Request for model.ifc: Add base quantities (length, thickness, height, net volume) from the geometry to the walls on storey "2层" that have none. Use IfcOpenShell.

First a look at what the model holds.

```python
import ifcopenshell
import ifcopenshell.util.element
import ifcopenshell.util.unit

model = ifcopenshell.open("model.ifc")
print(model.schema)
for unit_type in ("LENGTHUNIT", "AREAUNIT", "VOLUMEUNIT"):
    print(unit_type, ifcopenshell.util.unit.calculate_unit_scale(model, unit_type))
storey = next(s for s in model.by_type("IfcBuildingStorey") if s.Name == "2层")
walls = [e for e in ifcopenshell.util.element.get_decomposition(storey) if e.is_a("IfcWall")]
for e in sorted(walls, key=lambda e: e.id()):
    print(e.id(), e.is_a(), e.Name, list(ifcopenshell.util.element.get_psets(e, qtos_only=True)), sep=" | ")
```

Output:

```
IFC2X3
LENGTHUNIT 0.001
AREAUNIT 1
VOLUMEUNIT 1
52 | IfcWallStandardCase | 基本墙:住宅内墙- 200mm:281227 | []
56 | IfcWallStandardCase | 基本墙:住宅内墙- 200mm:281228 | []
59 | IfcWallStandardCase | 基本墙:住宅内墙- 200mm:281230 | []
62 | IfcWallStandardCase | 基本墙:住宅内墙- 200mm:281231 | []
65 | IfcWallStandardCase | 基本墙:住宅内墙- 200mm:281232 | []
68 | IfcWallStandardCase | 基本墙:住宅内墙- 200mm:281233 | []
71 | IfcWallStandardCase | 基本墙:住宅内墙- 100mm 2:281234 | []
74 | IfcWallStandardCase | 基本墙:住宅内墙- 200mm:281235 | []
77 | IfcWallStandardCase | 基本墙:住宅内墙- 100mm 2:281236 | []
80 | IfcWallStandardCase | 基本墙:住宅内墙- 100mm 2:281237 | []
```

```python
import ifcopenshell
import ifcopenshell.api.pset
import ifcopenshell.geom
import ifcopenshell.util.element
import ifcopenshell.util.shape
import ifcopenshell.util.unit

model = ifcopenshell.open("model.ifc")
unit_scale = ifcopenshell.util.unit.calculate_unit_scale(model)
volume_scale = ifcopenshell.util.unit.calculate_unit_scale(model, "VOLUMEUNIT")
settings = ifcopenshell.geom.settings()

storey = next(s for s in model.by_type("IfcBuildingStorey") if s.Name == "2层")
walls = [e for e in ifcopenshell.util.element.get_decomposition(storey) if e.is_a("IfcWall")]

for e in sorted(walls, key=lambda e: e.id()):
    if ifcopenshell.util.element.get_psets(e, qtos_only=True, should_inherit=False):
        continue
    # Geometry comes back in metres, in the element's own axes.
    shape = ifcopenshell.geom.create_shape(settings, e)
    values = {
        "Length": ifcopenshell.util.shape.get_x(shape.geometry) / unit_scale,
        "Width": ifcopenshell.util.shape.get_y(shape.geometry) / unit_scale,
        "Height": ifcopenshell.util.shape.get_z(shape.geometry) / unit_scale,
        "NetVolume": ifcopenshell.util.shape.get_volume(shape.geometry) / volume_scale,
    }
    qto = ifcopenshell.api.pset.add_qto(model, product=e, name="BaseQuantities")
    ifcopenshell.api.pset.edit_qto(model, qto=qto, properties=values)
    print(e.id(), {k: round(v, 3) for k, v in values.items()})

model.write("model_v2.ifc")
```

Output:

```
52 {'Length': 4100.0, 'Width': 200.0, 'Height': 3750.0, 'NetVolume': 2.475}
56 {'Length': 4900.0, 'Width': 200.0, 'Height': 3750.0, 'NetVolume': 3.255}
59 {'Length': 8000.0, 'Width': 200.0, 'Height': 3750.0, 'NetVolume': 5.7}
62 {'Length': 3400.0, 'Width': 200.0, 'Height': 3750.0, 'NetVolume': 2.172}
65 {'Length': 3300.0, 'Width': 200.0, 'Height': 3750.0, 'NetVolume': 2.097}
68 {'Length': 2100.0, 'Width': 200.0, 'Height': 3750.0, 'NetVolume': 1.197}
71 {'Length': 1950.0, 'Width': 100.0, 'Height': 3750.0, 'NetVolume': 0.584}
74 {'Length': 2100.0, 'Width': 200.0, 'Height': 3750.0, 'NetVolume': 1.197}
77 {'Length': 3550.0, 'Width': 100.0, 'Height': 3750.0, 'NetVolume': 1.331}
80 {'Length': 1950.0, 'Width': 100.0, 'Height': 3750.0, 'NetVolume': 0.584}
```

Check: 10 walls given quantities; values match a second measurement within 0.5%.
